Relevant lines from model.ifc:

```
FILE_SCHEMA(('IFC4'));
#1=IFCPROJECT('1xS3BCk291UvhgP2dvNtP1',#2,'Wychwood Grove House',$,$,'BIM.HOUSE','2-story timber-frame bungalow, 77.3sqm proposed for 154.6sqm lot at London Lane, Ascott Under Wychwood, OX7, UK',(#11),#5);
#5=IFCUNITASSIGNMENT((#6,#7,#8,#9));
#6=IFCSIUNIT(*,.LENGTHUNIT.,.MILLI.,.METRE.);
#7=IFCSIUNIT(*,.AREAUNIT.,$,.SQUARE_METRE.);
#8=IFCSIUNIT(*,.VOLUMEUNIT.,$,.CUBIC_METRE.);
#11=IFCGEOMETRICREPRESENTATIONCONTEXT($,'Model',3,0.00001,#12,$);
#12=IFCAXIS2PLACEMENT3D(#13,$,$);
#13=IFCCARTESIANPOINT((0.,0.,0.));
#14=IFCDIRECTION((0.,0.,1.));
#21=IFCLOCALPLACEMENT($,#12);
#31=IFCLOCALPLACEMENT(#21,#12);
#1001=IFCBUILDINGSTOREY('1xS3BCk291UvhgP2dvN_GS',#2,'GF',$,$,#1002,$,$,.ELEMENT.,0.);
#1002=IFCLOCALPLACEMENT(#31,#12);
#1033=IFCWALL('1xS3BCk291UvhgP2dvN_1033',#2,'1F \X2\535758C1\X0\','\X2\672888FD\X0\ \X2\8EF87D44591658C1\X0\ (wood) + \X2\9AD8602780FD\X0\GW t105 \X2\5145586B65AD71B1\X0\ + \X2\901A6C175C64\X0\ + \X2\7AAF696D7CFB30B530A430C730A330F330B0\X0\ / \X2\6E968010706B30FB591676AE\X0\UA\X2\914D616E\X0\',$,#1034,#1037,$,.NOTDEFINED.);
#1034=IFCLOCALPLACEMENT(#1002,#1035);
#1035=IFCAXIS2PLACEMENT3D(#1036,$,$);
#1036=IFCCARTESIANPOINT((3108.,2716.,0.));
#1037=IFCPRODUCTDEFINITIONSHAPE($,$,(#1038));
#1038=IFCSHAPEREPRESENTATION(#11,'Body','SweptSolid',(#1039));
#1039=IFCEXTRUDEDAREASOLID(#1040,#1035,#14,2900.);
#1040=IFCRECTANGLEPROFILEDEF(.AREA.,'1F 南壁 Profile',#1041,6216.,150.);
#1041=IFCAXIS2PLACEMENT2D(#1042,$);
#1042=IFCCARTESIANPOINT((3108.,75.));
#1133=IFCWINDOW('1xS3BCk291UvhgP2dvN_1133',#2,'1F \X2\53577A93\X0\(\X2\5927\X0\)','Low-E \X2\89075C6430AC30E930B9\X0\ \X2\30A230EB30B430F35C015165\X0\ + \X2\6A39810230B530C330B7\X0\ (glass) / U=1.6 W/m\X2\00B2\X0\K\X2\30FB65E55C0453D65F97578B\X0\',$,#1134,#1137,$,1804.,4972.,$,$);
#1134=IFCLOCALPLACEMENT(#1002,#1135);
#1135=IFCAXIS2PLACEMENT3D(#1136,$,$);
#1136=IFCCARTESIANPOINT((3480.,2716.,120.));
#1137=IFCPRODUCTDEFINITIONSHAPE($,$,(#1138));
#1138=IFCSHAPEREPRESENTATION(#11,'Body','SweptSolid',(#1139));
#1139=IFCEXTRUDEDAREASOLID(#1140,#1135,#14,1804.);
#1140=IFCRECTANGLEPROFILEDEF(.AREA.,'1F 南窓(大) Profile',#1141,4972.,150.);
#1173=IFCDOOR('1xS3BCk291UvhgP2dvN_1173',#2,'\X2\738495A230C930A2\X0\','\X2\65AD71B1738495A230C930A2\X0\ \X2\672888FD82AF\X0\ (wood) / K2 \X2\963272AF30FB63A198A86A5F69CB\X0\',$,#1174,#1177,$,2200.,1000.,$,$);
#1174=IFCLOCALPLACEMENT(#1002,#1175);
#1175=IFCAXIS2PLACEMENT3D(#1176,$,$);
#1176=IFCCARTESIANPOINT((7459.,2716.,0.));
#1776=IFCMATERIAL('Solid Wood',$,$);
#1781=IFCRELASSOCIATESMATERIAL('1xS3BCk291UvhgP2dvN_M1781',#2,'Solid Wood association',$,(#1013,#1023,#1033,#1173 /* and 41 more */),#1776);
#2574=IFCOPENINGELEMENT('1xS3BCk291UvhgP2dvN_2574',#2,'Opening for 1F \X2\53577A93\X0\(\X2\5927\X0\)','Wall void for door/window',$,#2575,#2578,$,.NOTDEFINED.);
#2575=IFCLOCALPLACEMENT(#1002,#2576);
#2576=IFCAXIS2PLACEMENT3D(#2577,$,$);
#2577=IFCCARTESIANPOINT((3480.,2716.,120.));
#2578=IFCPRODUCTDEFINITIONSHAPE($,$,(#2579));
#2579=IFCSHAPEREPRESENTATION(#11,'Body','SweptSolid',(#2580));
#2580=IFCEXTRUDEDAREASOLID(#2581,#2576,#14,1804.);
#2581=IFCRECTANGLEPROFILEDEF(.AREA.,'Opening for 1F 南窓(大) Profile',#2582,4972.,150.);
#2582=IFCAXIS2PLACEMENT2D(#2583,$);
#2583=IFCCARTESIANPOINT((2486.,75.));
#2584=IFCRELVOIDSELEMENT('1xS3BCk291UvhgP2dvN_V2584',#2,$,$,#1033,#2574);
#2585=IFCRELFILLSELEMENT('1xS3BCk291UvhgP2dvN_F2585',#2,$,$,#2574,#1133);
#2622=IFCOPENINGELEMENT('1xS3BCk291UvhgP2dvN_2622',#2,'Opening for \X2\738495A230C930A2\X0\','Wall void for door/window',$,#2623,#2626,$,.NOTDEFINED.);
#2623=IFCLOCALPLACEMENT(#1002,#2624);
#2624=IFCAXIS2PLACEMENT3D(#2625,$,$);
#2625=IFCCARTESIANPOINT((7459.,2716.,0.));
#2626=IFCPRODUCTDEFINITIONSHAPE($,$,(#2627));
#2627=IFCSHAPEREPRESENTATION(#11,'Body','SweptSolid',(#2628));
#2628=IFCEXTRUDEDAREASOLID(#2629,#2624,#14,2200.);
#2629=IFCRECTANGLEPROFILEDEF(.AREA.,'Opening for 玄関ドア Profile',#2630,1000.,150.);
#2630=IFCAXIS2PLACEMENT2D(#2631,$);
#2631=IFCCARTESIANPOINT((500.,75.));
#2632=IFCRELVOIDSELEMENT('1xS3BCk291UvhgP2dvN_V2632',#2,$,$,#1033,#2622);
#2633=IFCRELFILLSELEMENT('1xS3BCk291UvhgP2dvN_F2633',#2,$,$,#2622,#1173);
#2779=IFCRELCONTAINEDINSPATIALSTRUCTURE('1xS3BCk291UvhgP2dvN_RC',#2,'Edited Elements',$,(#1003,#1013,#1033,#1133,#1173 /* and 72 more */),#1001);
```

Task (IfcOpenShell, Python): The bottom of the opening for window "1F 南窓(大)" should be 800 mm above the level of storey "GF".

```python
import numpy as np
import ifcopenshell
import ifcopenshell.api.geometry
import ifcopenshell.geom
import ifcopenshell.util.element
import ifcopenshell.util.placement
import ifcopenshell.util.shape
import ifcopenshell.util.unit

model = ifcopenshell.open("model.ifc")
unit_scale = ifcopenshell.util.unit.calculate_unit_scale(model)

window = model.by_guid("1xS3BCk291UvhgP2dvN_1133")
opening = window.FillsVoids[0].RelatingOpeningElement
storey = ifcopenshell.util.element.get_container(window, ifc_class="IfcBuildingStorey")
level = ifcopenshell.util.placement.get_local_placement(storey.ObjectPlacement)[2, 3]

# The opening's origin need not be at the sill, so measure its lowest point.
shape = ifcopenshell.geom.create_shape(ifcopenshell.geom.settings(), opening)
bottom = ifcopenshell.util.shape.get_shape_bottom_elevation(shape, shape.geometry) / unit_scale
dz = level + 0.8 / unit_scale - bottom

shift = np.array([0.0, 0.0, dz])
# The window is not placed relative to its opening, so move both.
for product in (opening, window):
    matrix = ifcopenshell.util.placement.get_local_placement(product.ObjectPlacement)
    matrix[:3, 3] += shift
    ifcopenshell.api.geometry.edit_object_placement(model, product=product, matrix=matrix, is_si=False)

print(f"moved by {dz * unit_scale:+.3f} m")

model.write("model-out.ifc")
```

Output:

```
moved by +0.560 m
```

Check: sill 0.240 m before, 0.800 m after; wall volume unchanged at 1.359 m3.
